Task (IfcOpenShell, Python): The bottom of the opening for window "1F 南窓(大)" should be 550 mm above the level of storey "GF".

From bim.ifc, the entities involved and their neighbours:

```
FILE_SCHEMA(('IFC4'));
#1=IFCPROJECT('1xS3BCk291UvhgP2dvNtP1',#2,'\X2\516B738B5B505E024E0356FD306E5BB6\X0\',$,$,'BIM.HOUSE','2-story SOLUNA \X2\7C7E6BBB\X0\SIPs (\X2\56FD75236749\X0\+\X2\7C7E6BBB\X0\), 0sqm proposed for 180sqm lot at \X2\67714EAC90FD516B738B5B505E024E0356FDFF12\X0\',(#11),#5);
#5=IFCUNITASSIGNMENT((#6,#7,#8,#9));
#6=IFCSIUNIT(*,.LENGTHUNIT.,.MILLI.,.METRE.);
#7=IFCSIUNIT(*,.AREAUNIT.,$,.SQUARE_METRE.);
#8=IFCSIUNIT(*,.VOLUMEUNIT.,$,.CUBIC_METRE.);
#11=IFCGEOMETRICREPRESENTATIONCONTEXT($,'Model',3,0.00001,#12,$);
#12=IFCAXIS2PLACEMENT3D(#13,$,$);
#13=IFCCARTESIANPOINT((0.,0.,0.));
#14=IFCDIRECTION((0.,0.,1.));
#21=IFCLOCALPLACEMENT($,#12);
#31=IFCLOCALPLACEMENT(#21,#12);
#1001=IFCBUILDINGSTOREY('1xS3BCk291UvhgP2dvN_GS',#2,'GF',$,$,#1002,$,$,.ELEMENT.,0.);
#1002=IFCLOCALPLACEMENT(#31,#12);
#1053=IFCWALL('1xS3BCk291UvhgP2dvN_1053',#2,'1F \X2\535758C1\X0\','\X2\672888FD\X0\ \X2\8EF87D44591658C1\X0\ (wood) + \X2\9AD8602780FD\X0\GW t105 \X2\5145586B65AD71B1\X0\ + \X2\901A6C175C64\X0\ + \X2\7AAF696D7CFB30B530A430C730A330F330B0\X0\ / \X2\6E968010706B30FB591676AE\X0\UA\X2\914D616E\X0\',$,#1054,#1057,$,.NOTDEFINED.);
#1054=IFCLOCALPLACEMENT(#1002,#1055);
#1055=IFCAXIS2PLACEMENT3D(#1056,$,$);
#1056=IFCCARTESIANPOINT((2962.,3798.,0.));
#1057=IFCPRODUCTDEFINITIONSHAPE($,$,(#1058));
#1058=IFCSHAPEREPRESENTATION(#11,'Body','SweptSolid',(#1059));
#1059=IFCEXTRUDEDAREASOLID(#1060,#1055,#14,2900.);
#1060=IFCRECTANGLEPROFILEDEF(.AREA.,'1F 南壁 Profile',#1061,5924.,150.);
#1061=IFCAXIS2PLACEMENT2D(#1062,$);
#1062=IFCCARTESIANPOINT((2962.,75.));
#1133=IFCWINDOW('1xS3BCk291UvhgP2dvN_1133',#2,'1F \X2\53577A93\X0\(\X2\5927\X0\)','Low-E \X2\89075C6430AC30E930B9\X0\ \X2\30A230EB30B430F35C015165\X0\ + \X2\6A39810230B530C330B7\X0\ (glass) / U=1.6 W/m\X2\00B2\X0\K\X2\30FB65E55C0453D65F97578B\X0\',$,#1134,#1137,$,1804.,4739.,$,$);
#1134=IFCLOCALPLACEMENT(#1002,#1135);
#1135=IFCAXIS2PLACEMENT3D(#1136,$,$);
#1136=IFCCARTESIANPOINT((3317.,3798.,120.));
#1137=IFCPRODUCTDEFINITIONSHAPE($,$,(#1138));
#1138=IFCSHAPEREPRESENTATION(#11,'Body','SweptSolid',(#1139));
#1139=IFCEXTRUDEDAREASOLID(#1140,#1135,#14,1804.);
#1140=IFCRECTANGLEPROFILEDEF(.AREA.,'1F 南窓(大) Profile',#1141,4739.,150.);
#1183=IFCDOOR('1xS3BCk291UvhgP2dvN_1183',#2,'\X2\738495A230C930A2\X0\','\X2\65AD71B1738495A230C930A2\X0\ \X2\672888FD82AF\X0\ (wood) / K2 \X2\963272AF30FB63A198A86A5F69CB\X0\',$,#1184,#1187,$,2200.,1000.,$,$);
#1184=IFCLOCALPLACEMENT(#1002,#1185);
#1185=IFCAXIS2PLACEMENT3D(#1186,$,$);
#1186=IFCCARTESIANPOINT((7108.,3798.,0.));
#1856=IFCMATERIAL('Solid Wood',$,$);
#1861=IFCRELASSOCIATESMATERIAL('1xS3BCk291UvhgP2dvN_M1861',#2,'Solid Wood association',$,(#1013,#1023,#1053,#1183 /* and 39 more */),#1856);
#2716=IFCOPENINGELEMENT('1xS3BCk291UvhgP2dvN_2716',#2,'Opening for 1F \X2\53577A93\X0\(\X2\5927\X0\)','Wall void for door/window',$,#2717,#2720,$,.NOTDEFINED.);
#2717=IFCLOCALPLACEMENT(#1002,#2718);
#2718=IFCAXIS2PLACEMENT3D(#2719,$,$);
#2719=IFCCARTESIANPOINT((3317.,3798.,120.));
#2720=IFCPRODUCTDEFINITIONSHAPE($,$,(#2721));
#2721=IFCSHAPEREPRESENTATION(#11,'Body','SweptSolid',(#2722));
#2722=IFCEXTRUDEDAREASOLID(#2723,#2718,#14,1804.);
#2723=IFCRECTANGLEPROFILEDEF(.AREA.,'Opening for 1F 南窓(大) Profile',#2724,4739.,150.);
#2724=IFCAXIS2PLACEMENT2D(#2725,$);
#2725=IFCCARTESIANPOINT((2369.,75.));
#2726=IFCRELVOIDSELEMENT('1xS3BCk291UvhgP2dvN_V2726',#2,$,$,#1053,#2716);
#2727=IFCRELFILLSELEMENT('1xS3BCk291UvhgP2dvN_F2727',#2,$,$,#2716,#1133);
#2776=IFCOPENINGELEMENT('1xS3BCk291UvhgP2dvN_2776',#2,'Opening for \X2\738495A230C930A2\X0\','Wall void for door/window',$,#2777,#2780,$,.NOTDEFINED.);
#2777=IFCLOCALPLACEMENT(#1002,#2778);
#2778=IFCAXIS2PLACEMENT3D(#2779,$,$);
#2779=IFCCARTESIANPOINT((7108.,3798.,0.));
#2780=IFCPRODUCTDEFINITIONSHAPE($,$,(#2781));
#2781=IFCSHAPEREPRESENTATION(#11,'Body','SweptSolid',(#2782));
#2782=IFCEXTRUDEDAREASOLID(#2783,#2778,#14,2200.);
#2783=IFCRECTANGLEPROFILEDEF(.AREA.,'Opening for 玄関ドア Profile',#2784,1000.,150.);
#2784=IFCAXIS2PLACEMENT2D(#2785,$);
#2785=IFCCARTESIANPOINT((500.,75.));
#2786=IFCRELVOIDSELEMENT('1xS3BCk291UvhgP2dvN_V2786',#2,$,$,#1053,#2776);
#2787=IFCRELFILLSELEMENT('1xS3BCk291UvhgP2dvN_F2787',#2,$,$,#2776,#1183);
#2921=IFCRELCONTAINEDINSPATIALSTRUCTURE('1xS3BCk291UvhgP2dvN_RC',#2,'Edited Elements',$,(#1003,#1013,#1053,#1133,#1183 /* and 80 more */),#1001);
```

```python
import numpy as np
import ifcopenshell
import ifcopenshell.api.geometry
import ifcopenshell.geom
import ifcopenshell.util.element
import ifcopenshell.util.placement
import ifcopenshell.util.shape
import ifcopenshell.util.unit

model = ifcopenshell.open("bim.ifc")
unit_scale = ifcopenshell.util.unit.calculate_unit_scale(model)

window = model.by_guid("1xS3BCk291UvhgP2dvN_1133")
opening = window.FillsVoids[0].RelatingOpeningElement
storey = ifcopenshell.util.element.get_container(window, ifc_class="IfcBuildingStorey")
level = ifcopenshell.util.placement.get_local_placement(storey.ObjectPlacement)[2, 3]

# The opening's origin need not be at the sill, so measure its lowest point.
shape = ifcopenshell.geom.create_shape(ifcopenshell.geom.settings(), opening)
bottom = ifcopenshell.util.shape.get_shape_bottom_elevation(shape, shape.geometry) / unit_scale
dz = level + 0.55 / unit_scale - bottom

shift = np.array([0.0, 0.0, dz])
# The window is not placed relative to its opening, so move both.
for product in (opening, window):
    matrix = ifcopenshell.util.placement.get_local_placement(product.ObjectPlacement)
    matrix[:3, 3] += shift
    ifcopenshell.api.geometry.edit_object_placement(model, product=product, matrix=matrix, is_si=False)

print(f"moved by {dz * unit_scale:+.3f} m")

model.write("bim_rev.ifc")
```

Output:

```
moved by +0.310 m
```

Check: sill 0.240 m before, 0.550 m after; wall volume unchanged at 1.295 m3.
